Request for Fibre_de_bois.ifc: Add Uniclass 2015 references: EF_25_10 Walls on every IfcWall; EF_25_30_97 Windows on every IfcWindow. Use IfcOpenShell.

First a look at what the model holds.

```python
import ifcopenshell

model = ifcopenshell.open("Fibre_de_bois.ifc")
print(model.schema)
print("classifications:", [c.Name for c in model.by_type("IfcClassification")])
for ifc_class in ("IfcDoor", "IfcRoof", "IfcStair", "IfcWall", "IfcWindow"):
    print(ifc_class, len(model.by_type(ifc_class)))
```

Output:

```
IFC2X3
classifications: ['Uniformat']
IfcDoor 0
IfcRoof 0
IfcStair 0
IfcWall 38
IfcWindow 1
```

```python
import ifcopenshell
import ifcopenshell.api.classification

model = ifcopenshell.open("Fibre_de_bois.ifc")

# IFC2X3 requires Source and Edition and has no link from the project to the system.
system = model.create_entity("IfcClassification", Source="NBS", Edition="2015", Name="Uniclass 2015")

codes = {
    "IfcWall": ("EF_25_10", "Walls"),
    "IfcWindow": ("EF_25_30_97", "Windows"),
}
for ifc_class, (code, name) in codes.items():
    products = model.by_type(ifc_class)
    ifcopenshell.api.classification.add_reference(
        model, products=products, classification=system, identification=code, name=name
    )
    print(code, len(products))

model.write("Fibre_de_bois_edited.ifc")
```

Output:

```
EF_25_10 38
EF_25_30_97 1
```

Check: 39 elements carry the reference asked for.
